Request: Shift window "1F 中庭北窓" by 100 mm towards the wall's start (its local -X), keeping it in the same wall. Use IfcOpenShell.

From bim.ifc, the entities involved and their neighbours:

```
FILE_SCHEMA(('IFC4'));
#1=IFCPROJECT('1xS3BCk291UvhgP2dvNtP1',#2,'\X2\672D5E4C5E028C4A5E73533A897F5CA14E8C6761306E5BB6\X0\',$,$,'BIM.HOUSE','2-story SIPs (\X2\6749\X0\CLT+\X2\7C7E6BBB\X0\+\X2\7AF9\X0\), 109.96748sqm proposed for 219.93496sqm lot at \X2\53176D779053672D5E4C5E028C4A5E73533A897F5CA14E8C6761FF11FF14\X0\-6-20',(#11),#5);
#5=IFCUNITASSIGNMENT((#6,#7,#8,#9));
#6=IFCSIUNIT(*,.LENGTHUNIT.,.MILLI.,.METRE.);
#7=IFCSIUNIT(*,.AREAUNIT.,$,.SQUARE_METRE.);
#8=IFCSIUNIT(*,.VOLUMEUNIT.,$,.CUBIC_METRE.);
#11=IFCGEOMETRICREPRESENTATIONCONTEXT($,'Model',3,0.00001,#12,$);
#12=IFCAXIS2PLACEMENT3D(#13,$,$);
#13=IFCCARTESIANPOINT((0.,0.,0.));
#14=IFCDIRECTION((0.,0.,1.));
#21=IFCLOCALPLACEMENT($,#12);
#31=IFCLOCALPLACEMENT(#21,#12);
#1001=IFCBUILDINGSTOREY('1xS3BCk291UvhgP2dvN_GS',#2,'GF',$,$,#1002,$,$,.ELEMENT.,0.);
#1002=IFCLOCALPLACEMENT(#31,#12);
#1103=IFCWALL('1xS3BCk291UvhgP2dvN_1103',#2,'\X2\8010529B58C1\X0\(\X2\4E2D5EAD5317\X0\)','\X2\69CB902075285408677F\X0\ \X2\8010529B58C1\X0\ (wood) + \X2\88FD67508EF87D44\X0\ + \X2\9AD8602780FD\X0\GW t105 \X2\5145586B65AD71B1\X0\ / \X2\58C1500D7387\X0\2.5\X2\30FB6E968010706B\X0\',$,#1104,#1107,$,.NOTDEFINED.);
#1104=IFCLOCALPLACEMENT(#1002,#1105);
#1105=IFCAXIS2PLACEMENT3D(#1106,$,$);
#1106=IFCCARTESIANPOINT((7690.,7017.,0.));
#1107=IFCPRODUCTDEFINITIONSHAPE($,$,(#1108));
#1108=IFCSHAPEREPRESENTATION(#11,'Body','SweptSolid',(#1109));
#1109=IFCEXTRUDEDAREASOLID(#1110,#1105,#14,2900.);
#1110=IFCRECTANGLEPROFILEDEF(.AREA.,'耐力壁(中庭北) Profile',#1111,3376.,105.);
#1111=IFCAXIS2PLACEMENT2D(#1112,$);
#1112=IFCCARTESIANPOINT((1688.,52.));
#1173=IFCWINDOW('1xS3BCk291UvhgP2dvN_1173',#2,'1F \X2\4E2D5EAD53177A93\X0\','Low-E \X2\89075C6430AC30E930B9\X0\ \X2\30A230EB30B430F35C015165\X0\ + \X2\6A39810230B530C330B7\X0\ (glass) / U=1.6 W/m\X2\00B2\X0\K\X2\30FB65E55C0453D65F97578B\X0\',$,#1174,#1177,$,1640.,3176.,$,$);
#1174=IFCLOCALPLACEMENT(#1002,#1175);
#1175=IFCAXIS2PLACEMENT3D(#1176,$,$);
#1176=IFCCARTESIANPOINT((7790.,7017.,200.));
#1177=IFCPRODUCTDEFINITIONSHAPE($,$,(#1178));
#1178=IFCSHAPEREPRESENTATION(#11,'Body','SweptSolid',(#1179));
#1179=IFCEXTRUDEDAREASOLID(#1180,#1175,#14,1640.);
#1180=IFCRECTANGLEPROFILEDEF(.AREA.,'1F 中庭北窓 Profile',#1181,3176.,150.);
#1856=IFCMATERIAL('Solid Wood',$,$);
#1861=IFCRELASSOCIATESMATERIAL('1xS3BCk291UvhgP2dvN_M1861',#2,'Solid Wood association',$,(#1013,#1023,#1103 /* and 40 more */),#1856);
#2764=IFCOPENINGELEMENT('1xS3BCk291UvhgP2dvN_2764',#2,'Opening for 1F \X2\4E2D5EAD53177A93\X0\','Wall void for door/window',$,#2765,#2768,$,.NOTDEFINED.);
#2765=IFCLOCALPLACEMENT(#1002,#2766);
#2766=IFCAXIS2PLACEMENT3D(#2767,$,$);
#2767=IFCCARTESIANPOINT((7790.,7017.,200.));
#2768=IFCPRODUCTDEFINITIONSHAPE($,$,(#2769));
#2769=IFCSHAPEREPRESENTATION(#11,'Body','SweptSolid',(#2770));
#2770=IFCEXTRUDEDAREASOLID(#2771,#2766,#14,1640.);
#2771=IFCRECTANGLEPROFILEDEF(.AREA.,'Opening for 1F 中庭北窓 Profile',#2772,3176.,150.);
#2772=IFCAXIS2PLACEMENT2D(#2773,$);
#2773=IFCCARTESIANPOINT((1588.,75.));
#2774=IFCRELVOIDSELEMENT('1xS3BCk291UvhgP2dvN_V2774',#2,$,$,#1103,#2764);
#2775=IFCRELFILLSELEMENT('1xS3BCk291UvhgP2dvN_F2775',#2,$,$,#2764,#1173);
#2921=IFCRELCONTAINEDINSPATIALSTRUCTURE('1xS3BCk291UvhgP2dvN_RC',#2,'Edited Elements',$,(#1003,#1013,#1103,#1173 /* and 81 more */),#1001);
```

```python
import ifcopenshell
import ifcopenshell.api.geometry
import ifcopenshell.util.placement

model = ifcopenshell.open("bim.ifc")

window = model.by_guid("1xS3BCk291UvhgP2dvN_1173")
opening = window.FillsVoids[0].RelatingOpeningElement
wall = opening.VoidsElements[0].RelatingBuildingElement

wall_matrix = ifcopenshell.util.placement.get_local_placement(wall.ObjectPlacement)
shift = wall_matrix[:3, 0] * -100.0
before = ifcopenshell.util.placement.get_local_placement(window.ObjectPlacement)[:3, 3].copy()

# The window is not placed relative to its opening, so move both.
for product in (opening, window):
    matrix = ifcopenshell.util.placement.get_local_placement(product.ObjectPlacement)
    matrix[:3, 3] += shift
    ifcopenshell.api.geometry.edit_object_placement(model, product=product, matrix=matrix, is_si=False)

after = ifcopenshell.util.placement.get_local_placement(window.ObjectPlacement)[:3, 3]
print("window moved by", (after - before).round(3) + 0.0)

model.write("bim_updated.ifc")
```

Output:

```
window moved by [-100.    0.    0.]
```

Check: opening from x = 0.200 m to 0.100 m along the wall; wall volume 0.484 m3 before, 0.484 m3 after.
